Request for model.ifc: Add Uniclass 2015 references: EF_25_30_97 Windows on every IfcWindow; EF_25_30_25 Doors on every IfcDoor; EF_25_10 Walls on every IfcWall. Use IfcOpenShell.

First a look at what the model holds.

```python
import ifcopenshell

model = ifcopenshell.open("model.ifc")
print(model.schema)
print("classifications:", [c.Name for c in model.by_type("IfcClassification")])
for ifc_class in ("IfcDoor", "IfcRoof", "IfcStair", "IfcWall", "IfcWindow"):
    print(ifc_class, len(model.by_type(ifc_class)))
```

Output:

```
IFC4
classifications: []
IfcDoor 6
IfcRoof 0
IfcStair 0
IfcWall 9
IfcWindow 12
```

```python
import ifcopenshell
import ifcopenshell.api.classification

model = ifcopenshell.open("model.ifc")

system = ifcopenshell.api.classification.add_classification(model, classification="Uniclass 2015")

codes = {
    "IfcWindow": ("EF_25_30_97", "Windows"),
    "IfcDoor": ("EF_25_30_25", "Doors"),
    "IfcWall": ("EF_25_10", "Walls"),
}
for ifc_class, (code, name) in codes.items():
    products = model.by_type(ifc_class)
    ifcopenshell.api.classification.add_reference(
        model, products=products, classification=system, identification=code, name=name
    )
    print(code, len(products))

model.write("model_rev.ifc")
```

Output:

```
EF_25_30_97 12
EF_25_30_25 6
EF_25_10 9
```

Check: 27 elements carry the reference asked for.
